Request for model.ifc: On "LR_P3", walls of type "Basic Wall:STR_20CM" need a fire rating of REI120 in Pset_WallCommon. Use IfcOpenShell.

First a look at what the model holds.

```python
import ifcopenshell
import ifcopenshell.util.element

model = ifcopenshell.open("model.ifc")
print(model.schema)
storey = next(s for s in model.by_type("IfcBuildingStorey") if s.Name == "LR_P3")
walls = [e for e in ifcopenshell.util.element.get_decomposition(storey) if e.is_a("IfcWall")]
seen = {}
for e in walls:
    element_type = ifcopenshell.util.element.get_type(e)
    key = (element_type.Name if element_type != e and element_type else None, ifcopenshell.util.element.get_pset(e, "Pset_WallCommon", "FireRating"))
    seen[key] = seen.get(key, 0) + 1
for (name, value), count in sorted(seen.items(), key=str):
    print(count, "x", name, "|", value)
```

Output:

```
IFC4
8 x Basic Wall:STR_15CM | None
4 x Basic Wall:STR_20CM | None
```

```python
import ifcopenshell
import ifcopenshell.api.pset
import ifcopenshell.util.element

model = ifcopenshell.open("model.ifc")

storey = next(s for s in model.by_type("IfcBuildingStorey") if s.Name == "LR_P3")
walls = [e for e in ifcopenshell.util.element.get_decomposition(storey) if e.is_a("IfcWall")]

count = 0
for e in walls:
    element_type = ifcopenshell.util.element.get_type(e)
    if element_type in (None, e) or element_type.Name != "Basic Wall:STR_20CM":
        continue
    # add_pset returns the element's existing set when there is one.
    pset = ifcopenshell.api.pset.add_pset(model, product=e, name="Pset_WallCommon")
    ifcopenshell.api.pset.edit_pset(model, pset=pset, properties={"FireRating": "REI120"})
    count += 1

print(count, "walls updated")

model.write("model_edited.ifc")
```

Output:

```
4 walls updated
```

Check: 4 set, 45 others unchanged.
